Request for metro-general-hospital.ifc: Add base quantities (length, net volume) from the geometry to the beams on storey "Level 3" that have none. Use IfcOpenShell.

First a look at what the model holds.

```python
import ifcopenshell
import ifcopenshell.util.element
import ifcopenshell.util.unit

model = ifcopenshell.open("metro-general-hospital.ifc")
print(model.schema)
for unit_type in ("LENGTHUNIT", "AREAUNIT", "VOLUMEUNIT"):
    print(unit_type, ifcopenshell.util.unit.calculate_unit_scale(model, unit_type))
storey = next(s for s in model.by_type("IfcBuildingStorey") if s.Name == "Level 3")
beams = [e for e in ifcopenshell.util.element.get_decomposition(storey) if e.is_a("IfcBeam")]
for e in sorted(beams, key=lambda e: e.id()):
    print(e.id(), e.is_a(), e.Name, list(ifcopenshell.util.element.get_psets(e, qtos_only=True)), sep=" | ")
```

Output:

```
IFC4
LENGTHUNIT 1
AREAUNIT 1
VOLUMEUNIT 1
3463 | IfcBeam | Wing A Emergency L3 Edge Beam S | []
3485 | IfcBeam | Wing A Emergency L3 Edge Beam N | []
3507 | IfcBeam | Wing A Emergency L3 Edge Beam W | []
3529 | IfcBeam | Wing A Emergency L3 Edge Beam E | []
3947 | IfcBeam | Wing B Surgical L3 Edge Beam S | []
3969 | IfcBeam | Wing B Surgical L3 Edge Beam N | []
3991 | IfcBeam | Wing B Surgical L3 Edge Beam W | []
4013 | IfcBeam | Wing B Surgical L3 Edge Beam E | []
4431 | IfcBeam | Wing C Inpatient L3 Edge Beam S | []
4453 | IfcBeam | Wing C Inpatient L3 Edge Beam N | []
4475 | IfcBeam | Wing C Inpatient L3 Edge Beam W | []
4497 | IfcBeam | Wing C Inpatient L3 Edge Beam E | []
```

```python
import ifcopenshell
import ifcopenshell.api.pset
import ifcopenshell.geom
import ifcopenshell.util.element
import ifcopenshell.util.shape
import ifcopenshell.util.unit

model = ifcopenshell.open("metro-general-hospital.ifc")
unit_scale = ifcopenshell.util.unit.calculate_unit_scale(model)
volume_scale = ifcopenshell.util.unit.calculate_unit_scale(model, "VOLUMEUNIT")
settings = ifcopenshell.geom.settings()

storey = next(s for s in model.by_type("IfcBuildingStorey") if s.Name == "Level 3")
beams = [e for e in ifcopenshell.util.element.get_decomposition(storey) if e.is_a("IfcBeam")]

for e in sorted(beams, key=lambda e: e.id()):
    if ifcopenshell.util.element.get_psets(e, qtos_only=True, should_inherit=False):
        continue
    # Geometry comes back in metres, in the element's own axes.
    shape = ifcopenshell.geom.create_shape(settings, e)
    values = {
        "Length": ifcopenshell.util.shape.get_max_xyz(shape.geometry) / unit_scale,
        "NetVolume": ifcopenshell.util.shape.get_volume(shape.geometry) / volume_scale,
    }
    qto = ifcopenshell.api.pset.add_qto(model, product=e, name="Qto_BeamBaseQuantities")
    ifcopenshell.api.pset.edit_qto(model, qto=qto, properties=values)
    print(e.id(), {k: round(v, 3) for k, v in values.items()})

model.write("metro-general-hospital-out.ifc")
```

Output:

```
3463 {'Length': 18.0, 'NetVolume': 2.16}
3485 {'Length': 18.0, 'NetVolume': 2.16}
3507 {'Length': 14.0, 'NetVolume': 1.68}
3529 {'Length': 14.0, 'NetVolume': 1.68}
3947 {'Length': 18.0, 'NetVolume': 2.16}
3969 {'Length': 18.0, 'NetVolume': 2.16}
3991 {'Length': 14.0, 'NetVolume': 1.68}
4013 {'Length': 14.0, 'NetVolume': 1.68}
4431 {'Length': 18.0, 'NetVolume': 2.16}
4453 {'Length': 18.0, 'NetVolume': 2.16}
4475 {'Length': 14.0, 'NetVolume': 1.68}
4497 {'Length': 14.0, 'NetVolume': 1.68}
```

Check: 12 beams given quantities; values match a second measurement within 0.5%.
